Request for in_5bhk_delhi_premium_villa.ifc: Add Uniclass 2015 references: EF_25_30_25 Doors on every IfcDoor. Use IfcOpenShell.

First a look at what the model holds.

```python
import ifcopenshell

model = ifcopenshell.open("in_5bhk_delhi_premium_villa.ifc")
print(model.schema)
print("classifications:", [c.Name for c in model.by_type("IfcClassification")])
for ifc_class in ("IfcDoor", "IfcRoof", "IfcStair", "IfcWall", "IfcWindow"):
    print(ifc_class, len(model.by_type(ifc_class)))
```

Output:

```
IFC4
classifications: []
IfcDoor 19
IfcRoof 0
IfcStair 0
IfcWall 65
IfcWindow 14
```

```python
import ifcopenshell
import ifcopenshell.api.classification

model = ifcopenshell.open("in_5bhk_delhi_premium_villa.ifc")

system = ifcopenshell.api.classification.add_classification(model, classification="Uniclass 2015")

codes = {
    "IfcDoor": ("EF_25_30_25", "Doors"),
}
for ifc_class, (code, name) in codes.items():
    products = model.by_type(ifc_class)
    ifcopenshell.api.classification.add_reference(
        model, products=products, classification=system, identification=code, name=name
    )
    print(code, len(products))

model.write("in_5bhk_delhi_premium_villa_edited.ifc")
```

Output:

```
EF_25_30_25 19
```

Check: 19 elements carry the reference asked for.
